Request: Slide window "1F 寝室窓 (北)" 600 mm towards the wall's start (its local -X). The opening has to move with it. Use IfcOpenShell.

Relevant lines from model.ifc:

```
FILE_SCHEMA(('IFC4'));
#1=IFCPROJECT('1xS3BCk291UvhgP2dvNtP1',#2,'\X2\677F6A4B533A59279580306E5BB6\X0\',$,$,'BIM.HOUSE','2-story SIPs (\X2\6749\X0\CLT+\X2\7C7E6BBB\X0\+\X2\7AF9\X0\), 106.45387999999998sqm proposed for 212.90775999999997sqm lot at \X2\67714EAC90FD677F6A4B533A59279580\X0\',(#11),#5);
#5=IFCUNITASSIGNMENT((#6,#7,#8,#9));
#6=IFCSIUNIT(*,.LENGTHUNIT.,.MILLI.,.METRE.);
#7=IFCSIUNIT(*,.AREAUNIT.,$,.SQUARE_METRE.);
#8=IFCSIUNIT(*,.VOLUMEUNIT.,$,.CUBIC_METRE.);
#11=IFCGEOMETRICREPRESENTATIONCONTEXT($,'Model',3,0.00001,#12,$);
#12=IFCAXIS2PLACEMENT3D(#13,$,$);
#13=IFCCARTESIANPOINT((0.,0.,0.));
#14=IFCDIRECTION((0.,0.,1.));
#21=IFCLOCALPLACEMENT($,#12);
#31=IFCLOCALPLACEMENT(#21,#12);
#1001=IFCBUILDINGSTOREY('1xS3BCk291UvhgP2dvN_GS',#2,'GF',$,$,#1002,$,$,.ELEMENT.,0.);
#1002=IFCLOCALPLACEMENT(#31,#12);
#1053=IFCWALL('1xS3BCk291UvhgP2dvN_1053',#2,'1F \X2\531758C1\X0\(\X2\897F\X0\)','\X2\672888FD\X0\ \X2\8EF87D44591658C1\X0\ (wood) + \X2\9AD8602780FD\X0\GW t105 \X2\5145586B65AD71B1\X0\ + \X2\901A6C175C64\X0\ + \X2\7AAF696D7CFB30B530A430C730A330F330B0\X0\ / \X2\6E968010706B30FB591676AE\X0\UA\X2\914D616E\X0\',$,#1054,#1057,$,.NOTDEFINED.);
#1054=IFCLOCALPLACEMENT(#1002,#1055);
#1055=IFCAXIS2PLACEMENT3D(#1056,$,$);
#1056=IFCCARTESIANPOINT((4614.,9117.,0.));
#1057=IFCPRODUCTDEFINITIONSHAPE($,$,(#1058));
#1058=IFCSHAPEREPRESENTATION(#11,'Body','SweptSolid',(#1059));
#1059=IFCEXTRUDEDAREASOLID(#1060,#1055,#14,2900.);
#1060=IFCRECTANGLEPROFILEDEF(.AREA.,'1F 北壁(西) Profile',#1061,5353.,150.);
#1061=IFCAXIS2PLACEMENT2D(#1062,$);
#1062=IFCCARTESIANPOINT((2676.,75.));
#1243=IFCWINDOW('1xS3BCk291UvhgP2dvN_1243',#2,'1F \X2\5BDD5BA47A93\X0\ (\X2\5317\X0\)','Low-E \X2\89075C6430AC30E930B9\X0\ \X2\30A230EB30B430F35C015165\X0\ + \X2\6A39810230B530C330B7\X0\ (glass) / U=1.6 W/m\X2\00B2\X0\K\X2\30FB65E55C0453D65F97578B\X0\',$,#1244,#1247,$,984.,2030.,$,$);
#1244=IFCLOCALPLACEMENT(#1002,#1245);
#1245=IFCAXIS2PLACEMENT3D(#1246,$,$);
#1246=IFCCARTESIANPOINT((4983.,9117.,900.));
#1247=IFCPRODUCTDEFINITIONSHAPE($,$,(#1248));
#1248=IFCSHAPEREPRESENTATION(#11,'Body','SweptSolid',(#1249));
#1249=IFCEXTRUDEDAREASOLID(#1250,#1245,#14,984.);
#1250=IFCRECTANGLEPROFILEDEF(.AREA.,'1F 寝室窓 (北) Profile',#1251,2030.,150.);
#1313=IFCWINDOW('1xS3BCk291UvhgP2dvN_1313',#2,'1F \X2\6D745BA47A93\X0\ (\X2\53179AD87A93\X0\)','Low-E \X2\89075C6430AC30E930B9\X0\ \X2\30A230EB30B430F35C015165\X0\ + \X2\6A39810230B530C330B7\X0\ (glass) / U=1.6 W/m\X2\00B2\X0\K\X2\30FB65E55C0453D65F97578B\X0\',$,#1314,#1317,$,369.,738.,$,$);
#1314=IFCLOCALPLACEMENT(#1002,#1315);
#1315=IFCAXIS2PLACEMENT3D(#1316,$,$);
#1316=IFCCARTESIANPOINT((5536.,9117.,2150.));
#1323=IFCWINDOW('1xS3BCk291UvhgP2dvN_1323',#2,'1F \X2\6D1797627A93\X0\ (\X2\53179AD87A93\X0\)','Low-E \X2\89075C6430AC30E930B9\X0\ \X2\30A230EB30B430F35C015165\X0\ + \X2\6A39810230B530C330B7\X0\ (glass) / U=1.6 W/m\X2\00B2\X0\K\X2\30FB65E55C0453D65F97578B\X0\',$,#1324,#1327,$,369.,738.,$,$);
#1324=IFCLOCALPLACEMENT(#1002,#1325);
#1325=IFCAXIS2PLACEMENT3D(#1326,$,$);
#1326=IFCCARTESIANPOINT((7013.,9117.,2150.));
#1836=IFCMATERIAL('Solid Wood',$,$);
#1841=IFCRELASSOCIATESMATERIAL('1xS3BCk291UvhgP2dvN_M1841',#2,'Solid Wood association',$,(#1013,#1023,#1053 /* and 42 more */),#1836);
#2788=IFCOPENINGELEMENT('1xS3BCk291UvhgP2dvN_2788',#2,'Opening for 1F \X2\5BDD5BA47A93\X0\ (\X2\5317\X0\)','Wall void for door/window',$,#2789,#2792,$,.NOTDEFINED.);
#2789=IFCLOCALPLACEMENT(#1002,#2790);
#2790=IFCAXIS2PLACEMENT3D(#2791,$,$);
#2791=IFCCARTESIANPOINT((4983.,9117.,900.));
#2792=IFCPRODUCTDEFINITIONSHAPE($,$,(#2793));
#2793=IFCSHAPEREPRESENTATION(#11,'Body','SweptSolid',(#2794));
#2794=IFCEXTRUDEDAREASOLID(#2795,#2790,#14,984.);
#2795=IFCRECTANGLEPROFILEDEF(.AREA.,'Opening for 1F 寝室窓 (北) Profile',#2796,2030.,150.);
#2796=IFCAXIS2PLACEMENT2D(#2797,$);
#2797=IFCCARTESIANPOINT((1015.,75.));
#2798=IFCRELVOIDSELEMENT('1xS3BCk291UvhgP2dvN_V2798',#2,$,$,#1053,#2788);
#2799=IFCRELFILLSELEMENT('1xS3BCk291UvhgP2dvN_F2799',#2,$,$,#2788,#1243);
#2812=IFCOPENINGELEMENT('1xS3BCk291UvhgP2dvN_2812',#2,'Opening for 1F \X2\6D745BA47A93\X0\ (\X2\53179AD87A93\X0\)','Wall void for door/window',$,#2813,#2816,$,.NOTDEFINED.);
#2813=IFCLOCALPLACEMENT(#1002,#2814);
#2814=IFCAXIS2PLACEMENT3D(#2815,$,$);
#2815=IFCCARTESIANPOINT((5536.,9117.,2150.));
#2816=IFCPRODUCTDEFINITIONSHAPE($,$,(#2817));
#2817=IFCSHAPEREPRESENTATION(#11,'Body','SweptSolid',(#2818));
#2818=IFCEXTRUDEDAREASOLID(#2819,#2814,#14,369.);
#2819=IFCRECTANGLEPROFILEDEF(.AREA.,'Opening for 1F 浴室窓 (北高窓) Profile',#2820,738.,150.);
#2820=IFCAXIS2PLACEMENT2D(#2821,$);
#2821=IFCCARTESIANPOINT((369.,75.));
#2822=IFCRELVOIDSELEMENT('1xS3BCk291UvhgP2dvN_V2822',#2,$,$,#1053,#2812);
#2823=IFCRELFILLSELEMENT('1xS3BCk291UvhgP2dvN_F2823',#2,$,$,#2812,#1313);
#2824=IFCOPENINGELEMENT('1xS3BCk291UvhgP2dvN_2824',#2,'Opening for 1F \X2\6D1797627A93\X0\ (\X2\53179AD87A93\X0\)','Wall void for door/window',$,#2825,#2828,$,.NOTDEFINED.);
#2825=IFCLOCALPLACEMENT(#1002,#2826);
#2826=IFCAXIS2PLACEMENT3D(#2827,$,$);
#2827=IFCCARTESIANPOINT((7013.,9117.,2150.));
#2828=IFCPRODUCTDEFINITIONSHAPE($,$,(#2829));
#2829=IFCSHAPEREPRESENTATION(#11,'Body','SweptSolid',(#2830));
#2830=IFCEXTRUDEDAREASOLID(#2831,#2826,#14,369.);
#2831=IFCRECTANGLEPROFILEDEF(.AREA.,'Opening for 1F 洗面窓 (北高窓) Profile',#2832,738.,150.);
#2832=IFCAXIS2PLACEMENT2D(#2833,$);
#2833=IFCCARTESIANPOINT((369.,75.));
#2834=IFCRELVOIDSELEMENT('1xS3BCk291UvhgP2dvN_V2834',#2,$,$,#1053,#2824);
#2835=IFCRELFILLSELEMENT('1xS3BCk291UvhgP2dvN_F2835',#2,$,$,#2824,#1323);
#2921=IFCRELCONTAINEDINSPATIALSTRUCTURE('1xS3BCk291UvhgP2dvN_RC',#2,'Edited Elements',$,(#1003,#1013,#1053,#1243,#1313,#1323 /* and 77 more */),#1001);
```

```python
import ifcopenshell
import ifcopenshell.api.geometry
import ifcopenshell.util.placement
import ifcopenshell.util.unit

model = ifcopenshell.open("model.ifc")
unit_scale = ifcopenshell.util.unit.calculate_unit_scale(model)

window = model.by_id(1243)
opening = window.FillsVoids[0].RelatingOpeningElement
wall = opening.VoidsElements[0].RelatingBuildingElement

wall_matrix = ifcopenshell.util.placement.get_local_placement(wall.ObjectPlacement)
shift = wall_matrix[:3, 0] * -0.6 / unit_scale
before = ifcopenshell.util.placement.get_local_placement(window.ObjectPlacement)[:3, 3].copy()

# The window is not placed relative to its opening, so move both.
for product in (opening, window):
    matrix = ifcopenshell.util.placement.get_local_placement(product.ObjectPlacement)
    matrix[:3, 3] += shift
    ifcopenshell.api.geometry.edit_object_placement(model, product=product, matrix=matrix, is_si=False)

after = ifcopenshell.util.placement.get_local_placement(window.ObjectPlacement)[:3, 3]
print("window moved by", (after - before).round(3) + 0.0)

model.write("model_rev.ifc")
```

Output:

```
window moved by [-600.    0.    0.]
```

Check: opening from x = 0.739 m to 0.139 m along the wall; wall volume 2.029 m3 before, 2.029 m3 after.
